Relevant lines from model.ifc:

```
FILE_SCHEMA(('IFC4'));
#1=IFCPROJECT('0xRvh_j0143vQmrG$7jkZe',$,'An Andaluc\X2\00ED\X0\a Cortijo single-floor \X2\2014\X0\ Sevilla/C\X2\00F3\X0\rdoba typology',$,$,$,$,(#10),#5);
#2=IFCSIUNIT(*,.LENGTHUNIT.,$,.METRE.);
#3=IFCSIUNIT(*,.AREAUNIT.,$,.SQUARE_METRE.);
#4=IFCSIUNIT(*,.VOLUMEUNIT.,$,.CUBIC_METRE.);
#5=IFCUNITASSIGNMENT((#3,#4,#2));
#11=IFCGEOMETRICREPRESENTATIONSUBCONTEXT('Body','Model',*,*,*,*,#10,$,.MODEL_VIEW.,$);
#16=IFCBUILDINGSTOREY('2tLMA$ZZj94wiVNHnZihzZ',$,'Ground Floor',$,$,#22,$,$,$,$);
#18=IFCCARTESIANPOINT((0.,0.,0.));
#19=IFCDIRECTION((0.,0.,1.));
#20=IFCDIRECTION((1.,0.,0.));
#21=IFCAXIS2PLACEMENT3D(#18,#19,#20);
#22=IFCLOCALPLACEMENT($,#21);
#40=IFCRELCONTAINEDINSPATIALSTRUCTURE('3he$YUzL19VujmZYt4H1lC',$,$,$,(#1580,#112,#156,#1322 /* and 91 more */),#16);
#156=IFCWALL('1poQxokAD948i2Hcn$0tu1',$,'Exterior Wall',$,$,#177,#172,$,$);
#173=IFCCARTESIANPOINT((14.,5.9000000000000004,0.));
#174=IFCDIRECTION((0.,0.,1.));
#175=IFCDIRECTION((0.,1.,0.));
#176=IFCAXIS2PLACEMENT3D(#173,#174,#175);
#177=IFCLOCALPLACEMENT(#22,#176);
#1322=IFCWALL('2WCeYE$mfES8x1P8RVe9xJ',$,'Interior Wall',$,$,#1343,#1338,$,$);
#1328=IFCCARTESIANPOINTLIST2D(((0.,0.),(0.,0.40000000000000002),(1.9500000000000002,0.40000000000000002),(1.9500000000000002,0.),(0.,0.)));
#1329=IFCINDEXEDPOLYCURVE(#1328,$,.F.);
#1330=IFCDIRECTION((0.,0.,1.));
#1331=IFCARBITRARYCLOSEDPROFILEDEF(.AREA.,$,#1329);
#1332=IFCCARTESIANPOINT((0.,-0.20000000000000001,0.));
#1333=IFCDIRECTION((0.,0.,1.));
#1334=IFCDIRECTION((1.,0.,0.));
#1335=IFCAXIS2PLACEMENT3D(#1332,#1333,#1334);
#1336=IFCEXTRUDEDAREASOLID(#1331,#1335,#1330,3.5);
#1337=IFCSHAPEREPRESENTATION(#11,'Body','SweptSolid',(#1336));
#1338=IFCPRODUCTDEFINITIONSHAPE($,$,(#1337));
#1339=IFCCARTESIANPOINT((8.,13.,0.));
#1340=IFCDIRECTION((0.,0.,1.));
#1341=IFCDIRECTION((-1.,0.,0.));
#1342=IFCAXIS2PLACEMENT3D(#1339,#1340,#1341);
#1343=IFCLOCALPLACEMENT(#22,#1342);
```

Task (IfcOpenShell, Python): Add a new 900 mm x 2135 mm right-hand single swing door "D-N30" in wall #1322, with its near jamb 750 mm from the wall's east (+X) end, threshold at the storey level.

```python
import numpy as np
import ifcopenshell
import ifcopenshell.api.feature
import ifcopenshell.api.geometry
import ifcopenshell.api.root
import ifcopenshell.api.spatial
import ifcopenshell.geom
import ifcopenshell.util.element
import ifcopenshell.util.placement
import ifcopenshell.util.representation
import ifcopenshell.util.shape
import ifcopenshell.util.unit

model = ifcopenshell.open("model.ifc")
unit_scale = ifcopenshell.util.unit.calculate_unit_scale(model)
settings = ifcopenshell.geom.settings()


def volume(element):
    """Net volume in cubic metres, openings subtracted."""
    shape = ifcopenshell.geom.create_shape(settings, element)
    return ifcopenshell.util.shape.get_volume(shape.geometry)


wall = model.by_guid("2WCeYE$mfES8x1P8RVe9xJ")
storey = ifcopenshell.util.element.get_container(wall, ifc_class="IfcBuildingStorey")
context = ifcopenshell.util.representation.get_context(model, "Model", "Body", "MODEL_VIEW")
before = volume(wall)

width, height, from_end, sill = 0.9, 2.135, 0.75, 0.0  # metres

# The wall runs along its own X axis, and the end named is its -X end.
wall_shape = ifcopenshell.geom.create_shape(settings, wall)
x, y, z = ifcopenshell.util.shape.get_vertices(wall_shape.geometry).T
start = x.min() + from_end
face, thickness = float(y.min()), float(y.max() - y.min())
wall_matrix = ifcopenshell.util.placement.get_local_placement(wall.ObjectPlacement)
level = ifcopenshell.util.placement.get_local_placement(storey.ObjectPlacement)[2, 3]


def in_wall(x, y):
    """Placement at x, y metres in the wall's axes, at sill height."""
    matrix = wall_matrix.copy()
    matrix[:, 3] = wall_matrix @ np.array([x / unit_scale, y / unit_scale, 0.0, 1.0])
    matrix[2, 3] = level + sill / unit_scale
    return matrix


# Opening: a box that overshoots both wall faces by 50 mm.
opening = ifcopenshell.api.root.create_entity(model, ifc_class="IfcOpeningElement", predefined_type="OPENING")
box = ifcopenshell.api.geometry.add_wall_representation(
    model, context=context, length=width, height=height, thickness=thickness + 0.1
)
ifcopenshell.api.geometry.assign_representation(model, product=opening, representation=box)
ifcopenshell.api.geometry.edit_object_placement(model, product=opening, matrix=in_wall(start, face - 0.05), is_si=False)
ifcopenshell.api.feature.add_feature(model, feature=opening, element=wall)

door = ifcopenshell.api.root.create_entity(model, ifc_class="IfcDoor", name="D-N30", predefined_type="DOOR")
door.OverallWidth, door.OverallHeight = width / unit_scale, height / unit_scale
door.OperationType = "SINGLE_SWING_RIGHT"
body = ifcopenshell.api.geometry.add_door_representation(
    model,
    context=context,
    overall_width=door.OverallWidth,
    overall_height=door.OverallHeight,
    operation_type="SINGLE_SWING_RIGHT",
    lining_properties={"LiningDepth": thickness / unit_scale, "ThresholdDepth": thickness / unit_scale},
)
ifcopenshell.api.geometry.assign_representation(model, product=door, representation=body)
ifcopenshell.api.spatial.assign_container(model, products=[door], relating_structure=storey)
ifcopenshell.api.feature.add_filling(model, opening=opening, element=door)

# The lining spans the wall, so the door starts at the wall face.
ifcopenshell.api.geometry.edit_object_placement(model, product=door, matrix=in_wall(start, face), is_si=False)

after = volume(wall)

print(f"wall volume {before:.3f} -> {after:.3f} m3")

model.write("model_updated.ifc")
```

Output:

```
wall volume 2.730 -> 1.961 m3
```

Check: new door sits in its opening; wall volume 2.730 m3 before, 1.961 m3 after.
